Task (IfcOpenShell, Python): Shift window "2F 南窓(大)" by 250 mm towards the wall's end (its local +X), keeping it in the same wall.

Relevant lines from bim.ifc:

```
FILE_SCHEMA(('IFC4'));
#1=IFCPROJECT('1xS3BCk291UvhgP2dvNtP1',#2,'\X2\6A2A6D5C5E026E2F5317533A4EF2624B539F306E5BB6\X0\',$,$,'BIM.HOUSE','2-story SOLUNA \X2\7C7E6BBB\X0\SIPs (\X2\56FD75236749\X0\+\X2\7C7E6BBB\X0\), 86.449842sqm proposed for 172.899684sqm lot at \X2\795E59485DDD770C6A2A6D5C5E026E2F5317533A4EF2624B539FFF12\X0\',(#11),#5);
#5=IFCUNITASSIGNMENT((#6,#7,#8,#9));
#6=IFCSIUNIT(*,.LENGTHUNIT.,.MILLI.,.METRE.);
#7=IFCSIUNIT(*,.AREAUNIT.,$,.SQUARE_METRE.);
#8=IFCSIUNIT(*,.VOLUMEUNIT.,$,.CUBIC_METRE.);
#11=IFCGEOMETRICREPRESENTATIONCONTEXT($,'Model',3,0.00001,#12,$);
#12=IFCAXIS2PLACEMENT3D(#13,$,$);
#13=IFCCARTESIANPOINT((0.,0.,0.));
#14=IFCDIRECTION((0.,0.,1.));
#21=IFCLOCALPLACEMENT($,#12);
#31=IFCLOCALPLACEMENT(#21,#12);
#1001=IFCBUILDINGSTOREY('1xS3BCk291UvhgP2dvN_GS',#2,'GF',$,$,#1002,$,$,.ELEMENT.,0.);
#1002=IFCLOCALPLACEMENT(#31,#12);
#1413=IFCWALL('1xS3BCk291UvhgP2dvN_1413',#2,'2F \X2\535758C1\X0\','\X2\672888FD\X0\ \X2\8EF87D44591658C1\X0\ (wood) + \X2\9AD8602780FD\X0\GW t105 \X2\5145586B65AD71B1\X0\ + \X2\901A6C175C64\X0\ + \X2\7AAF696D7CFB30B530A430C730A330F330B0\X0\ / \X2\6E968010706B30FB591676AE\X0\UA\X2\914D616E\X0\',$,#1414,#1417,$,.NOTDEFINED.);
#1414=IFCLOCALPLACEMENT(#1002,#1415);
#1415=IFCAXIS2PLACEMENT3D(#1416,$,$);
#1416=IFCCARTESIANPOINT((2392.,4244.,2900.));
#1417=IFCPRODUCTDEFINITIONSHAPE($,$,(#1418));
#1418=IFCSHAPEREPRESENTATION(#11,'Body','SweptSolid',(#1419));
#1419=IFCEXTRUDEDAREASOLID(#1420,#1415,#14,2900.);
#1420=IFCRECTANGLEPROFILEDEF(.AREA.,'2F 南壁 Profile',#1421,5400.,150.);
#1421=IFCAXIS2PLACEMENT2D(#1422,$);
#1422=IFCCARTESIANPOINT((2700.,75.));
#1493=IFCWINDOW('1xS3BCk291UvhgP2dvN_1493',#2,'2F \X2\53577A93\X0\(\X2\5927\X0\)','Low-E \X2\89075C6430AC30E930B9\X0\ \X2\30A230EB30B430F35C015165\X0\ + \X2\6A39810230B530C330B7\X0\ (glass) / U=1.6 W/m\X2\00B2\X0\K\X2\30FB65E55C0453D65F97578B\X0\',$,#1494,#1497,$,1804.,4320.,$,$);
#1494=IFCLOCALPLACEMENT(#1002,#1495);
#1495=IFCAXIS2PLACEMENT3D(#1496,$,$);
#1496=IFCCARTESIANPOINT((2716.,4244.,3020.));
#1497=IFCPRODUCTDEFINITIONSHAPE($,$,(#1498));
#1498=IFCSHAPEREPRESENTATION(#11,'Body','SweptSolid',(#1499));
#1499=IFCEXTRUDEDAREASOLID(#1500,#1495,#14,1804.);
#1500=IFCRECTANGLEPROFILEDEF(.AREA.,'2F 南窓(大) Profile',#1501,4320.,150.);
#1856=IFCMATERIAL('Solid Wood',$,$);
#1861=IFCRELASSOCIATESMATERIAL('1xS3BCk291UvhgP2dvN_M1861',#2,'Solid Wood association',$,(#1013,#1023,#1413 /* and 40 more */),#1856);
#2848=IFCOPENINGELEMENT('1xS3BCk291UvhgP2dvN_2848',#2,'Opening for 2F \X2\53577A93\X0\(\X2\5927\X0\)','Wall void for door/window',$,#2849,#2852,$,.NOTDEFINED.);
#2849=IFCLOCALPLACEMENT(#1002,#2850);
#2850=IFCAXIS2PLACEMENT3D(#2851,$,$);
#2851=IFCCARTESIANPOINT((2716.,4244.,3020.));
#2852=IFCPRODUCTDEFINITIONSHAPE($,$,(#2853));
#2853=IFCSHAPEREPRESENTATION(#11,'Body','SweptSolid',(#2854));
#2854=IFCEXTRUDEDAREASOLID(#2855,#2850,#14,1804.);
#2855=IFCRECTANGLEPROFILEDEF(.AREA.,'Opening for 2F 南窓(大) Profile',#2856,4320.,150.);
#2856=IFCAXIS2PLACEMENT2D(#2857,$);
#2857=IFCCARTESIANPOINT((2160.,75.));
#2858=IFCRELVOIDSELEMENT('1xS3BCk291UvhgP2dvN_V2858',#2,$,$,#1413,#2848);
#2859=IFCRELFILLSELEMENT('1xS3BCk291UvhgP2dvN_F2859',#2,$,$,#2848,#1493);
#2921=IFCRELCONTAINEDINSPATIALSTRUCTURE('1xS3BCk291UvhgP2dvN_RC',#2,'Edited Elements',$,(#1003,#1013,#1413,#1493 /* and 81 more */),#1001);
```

```python
import ifcopenshell
import ifcopenshell.api.geometry
import ifcopenshell.util.placement
import ifcopenshell.util.unit

model = ifcopenshell.open("bim.ifc")
unit_scale = ifcopenshell.util.unit.calculate_unit_scale(model)

window = model.by_id(1493)
opening = window.FillsVoids[0].RelatingOpeningElement
wall = opening.VoidsElements[0].RelatingBuildingElement

wall_matrix = ifcopenshell.util.placement.get_local_placement(wall.ObjectPlacement)
shift = wall_matrix[:3, 0] * 0.25 / unit_scale
before = ifcopenshell.util.placement.get_local_placement(window.ObjectPlacement)[:3, 3].copy()

# The window is not placed relative to its opening, so move both.
for product in (opening, window):
    matrix = ifcopenshell.util.placement.get_local_placement(product.ObjectPlacement)
    matrix[:3, 3] += shift
    ifcopenshell.api.geometry.edit_object_placement(model, product=product, matrix=matrix, is_si=False)

after = ifcopenshell.util.placement.get_local_placement(window.ObjectPlacement)[:3, 3]
print("window moved by", (after - before).round(3) + 0.0)

model.write("bim_edited.ifc")
```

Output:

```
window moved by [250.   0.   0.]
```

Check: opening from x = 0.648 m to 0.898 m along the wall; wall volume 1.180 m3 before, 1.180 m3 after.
